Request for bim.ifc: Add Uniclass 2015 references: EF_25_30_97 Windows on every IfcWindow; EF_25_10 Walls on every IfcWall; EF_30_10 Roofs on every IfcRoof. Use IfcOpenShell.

First a look at what the model holds.

```python
import ifcopenshell

model = ifcopenshell.open("bim.ifc")
print(model.schema)
print("classifications:", [c.Name for c in model.by_type("IfcClassification")])
for ifc_class in ("IfcDoor", "IfcRoof", "IfcStair", "IfcWall", "IfcWindow"):
    print(ifc_class, len(model.by_type(ifc_class)))
```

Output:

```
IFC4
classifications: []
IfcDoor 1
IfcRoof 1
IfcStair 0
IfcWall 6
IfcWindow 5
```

```python
import ifcopenshell
import ifcopenshell.api.classification

model = ifcopenshell.open("bim.ifc")

system = ifcopenshell.api.classification.add_classification(model, classification="Uniclass 2015")

codes = {
    "IfcWindow": ("EF_25_30_97", "Windows"),
    "IfcWall": ("EF_25_10", "Walls"),
    "IfcRoof": ("EF_30_10", "Roofs"),
}
for ifc_class, (code, name) in codes.items():
    products = model.by_type(ifc_class)
    ifcopenshell.api.classification.add_reference(
        model, products=products, classification=system, identification=code, name=name
    )
    print(code, len(products))

model.write("bim_rev.ifc")
```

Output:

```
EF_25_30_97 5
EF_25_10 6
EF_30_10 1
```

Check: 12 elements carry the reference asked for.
